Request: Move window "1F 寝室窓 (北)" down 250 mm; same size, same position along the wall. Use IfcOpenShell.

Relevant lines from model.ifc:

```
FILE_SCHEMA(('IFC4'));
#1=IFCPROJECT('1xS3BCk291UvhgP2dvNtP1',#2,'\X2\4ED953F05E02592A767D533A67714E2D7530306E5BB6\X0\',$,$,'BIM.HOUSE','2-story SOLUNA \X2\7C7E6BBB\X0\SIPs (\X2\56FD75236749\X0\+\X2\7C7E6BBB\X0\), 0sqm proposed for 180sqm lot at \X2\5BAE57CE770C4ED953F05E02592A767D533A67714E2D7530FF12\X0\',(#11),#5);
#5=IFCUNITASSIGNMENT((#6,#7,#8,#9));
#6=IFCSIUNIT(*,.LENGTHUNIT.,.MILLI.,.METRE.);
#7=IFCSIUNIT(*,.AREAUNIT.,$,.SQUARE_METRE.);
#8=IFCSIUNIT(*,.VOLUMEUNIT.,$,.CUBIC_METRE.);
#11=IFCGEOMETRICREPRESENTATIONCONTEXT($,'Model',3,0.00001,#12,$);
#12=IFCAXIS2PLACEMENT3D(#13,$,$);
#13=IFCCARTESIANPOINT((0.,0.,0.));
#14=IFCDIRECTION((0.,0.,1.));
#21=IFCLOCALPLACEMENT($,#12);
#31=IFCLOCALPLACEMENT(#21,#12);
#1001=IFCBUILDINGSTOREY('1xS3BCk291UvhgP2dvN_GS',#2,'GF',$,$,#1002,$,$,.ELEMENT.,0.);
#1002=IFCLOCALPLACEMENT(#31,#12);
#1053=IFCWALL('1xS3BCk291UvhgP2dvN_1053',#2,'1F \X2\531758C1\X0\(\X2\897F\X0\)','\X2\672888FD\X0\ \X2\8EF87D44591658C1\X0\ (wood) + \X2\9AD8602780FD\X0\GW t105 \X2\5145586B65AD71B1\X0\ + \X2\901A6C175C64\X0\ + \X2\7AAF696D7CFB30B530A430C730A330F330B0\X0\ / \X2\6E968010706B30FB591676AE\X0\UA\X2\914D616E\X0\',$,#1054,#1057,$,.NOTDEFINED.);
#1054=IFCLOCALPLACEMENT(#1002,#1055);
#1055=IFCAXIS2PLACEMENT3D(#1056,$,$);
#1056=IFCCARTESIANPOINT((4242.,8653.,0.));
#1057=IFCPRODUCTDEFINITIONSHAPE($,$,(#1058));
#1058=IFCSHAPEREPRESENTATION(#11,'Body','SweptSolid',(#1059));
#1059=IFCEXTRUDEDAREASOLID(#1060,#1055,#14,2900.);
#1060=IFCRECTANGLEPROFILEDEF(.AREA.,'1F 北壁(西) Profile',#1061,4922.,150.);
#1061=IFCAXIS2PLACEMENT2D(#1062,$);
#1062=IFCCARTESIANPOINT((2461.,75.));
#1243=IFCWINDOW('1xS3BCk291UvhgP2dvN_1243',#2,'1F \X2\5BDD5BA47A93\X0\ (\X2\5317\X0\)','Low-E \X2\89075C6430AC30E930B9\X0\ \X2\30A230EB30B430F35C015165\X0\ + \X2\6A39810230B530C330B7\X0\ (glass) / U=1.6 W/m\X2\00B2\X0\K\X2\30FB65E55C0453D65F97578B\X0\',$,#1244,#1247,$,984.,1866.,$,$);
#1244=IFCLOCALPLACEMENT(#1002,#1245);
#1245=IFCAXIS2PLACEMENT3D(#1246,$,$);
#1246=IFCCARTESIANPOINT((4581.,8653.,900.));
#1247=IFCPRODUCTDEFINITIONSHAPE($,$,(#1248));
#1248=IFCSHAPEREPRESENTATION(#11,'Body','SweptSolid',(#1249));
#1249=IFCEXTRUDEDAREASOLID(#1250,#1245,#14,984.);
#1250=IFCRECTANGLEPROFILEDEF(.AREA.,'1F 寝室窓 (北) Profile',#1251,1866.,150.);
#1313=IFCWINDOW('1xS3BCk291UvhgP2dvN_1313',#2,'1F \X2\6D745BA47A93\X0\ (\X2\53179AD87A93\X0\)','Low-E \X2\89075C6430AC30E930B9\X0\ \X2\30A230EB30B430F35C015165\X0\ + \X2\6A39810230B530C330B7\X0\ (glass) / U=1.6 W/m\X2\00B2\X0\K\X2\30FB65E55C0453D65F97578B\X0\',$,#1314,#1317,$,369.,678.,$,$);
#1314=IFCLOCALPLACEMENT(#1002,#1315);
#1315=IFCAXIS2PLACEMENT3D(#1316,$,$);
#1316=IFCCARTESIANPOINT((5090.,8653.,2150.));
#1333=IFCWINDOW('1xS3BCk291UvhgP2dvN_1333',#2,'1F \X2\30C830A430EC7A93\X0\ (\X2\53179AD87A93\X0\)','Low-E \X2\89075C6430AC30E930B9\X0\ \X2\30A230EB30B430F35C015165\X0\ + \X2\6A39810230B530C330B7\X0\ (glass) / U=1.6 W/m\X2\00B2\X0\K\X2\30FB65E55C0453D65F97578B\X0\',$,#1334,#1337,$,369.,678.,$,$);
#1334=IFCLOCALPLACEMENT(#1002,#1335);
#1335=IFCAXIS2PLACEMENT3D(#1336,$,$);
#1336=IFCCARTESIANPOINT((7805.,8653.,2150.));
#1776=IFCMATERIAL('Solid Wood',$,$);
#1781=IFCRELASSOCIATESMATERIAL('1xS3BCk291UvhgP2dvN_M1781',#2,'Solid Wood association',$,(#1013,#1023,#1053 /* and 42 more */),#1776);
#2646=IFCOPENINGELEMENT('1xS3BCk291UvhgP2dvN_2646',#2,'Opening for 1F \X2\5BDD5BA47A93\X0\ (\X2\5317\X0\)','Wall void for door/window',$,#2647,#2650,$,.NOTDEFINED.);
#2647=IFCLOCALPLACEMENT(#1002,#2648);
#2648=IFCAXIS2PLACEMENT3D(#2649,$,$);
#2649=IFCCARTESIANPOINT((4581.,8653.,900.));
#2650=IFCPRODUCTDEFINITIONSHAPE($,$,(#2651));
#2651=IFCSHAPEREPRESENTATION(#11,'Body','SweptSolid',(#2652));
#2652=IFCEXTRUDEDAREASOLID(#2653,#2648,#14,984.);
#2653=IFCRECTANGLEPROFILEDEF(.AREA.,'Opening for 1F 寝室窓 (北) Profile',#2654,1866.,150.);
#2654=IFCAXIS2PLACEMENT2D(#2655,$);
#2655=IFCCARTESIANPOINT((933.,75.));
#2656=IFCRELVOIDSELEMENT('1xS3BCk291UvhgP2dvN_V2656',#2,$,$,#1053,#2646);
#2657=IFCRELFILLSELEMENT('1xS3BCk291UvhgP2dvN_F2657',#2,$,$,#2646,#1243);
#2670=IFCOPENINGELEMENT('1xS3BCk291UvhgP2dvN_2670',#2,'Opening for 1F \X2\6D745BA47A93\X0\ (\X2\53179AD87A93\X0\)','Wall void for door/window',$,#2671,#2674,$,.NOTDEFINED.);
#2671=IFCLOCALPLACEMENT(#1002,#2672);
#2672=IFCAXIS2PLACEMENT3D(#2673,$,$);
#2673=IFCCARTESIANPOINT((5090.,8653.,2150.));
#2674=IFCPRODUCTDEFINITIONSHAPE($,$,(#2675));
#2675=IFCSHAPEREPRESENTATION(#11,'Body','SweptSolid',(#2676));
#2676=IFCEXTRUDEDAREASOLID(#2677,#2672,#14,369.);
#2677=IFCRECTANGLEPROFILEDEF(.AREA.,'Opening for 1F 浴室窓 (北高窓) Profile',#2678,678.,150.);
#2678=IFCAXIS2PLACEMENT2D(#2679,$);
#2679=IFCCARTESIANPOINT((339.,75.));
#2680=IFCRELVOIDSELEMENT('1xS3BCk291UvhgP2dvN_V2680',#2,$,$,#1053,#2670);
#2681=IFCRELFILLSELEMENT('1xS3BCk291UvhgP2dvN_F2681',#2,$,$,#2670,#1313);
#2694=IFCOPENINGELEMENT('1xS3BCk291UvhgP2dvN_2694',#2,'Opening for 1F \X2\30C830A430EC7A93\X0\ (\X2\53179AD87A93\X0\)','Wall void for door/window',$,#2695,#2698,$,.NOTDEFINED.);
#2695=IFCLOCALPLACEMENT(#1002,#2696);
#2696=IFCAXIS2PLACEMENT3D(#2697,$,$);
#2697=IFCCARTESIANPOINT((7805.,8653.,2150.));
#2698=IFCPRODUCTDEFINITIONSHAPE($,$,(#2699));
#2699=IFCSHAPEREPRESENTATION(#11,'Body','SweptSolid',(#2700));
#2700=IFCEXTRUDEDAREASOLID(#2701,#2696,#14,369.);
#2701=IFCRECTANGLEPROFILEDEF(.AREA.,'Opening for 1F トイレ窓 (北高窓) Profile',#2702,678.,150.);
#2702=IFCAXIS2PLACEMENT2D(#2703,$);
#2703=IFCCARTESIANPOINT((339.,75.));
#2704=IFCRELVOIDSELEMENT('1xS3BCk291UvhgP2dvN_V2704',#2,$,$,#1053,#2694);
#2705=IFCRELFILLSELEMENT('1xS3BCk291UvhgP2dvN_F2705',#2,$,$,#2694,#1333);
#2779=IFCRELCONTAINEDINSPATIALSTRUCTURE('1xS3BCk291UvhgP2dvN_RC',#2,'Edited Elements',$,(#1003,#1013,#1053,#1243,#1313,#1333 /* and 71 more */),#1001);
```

```python
import numpy as np
import ifcopenshell
import ifcopenshell.api.geometry
import ifcopenshell.util.placement
import ifcopenshell.util.unit

model = ifcopenshell.open("model.ifc")
unit_scale = ifcopenshell.util.unit.calculate_unit_scale(model)

window = model.by_guid("1xS3BCk291UvhgP2dvN_1243")
opening = window.FillsVoids[0].RelatingOpeningElement
dz = -250.0

shift = np.array([0.0, 0.0, dz])
# The window is not placed relative to its opening, so move both.
for product in (opening, window):
    matrix = ifcopenshell.util.placement.get_local_placement(product.ObjectPlacement)
    matrix[:3, 3] += shift
    ifcopenshell.api.geometry.edit_object_placement(model, product=product, matrix=matrix, is_si=False)

print(f"moved by {dz * unit_scale:+.3f} m")

model.write("model_edited.ifc")
```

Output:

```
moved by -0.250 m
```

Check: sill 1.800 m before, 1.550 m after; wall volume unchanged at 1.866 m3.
